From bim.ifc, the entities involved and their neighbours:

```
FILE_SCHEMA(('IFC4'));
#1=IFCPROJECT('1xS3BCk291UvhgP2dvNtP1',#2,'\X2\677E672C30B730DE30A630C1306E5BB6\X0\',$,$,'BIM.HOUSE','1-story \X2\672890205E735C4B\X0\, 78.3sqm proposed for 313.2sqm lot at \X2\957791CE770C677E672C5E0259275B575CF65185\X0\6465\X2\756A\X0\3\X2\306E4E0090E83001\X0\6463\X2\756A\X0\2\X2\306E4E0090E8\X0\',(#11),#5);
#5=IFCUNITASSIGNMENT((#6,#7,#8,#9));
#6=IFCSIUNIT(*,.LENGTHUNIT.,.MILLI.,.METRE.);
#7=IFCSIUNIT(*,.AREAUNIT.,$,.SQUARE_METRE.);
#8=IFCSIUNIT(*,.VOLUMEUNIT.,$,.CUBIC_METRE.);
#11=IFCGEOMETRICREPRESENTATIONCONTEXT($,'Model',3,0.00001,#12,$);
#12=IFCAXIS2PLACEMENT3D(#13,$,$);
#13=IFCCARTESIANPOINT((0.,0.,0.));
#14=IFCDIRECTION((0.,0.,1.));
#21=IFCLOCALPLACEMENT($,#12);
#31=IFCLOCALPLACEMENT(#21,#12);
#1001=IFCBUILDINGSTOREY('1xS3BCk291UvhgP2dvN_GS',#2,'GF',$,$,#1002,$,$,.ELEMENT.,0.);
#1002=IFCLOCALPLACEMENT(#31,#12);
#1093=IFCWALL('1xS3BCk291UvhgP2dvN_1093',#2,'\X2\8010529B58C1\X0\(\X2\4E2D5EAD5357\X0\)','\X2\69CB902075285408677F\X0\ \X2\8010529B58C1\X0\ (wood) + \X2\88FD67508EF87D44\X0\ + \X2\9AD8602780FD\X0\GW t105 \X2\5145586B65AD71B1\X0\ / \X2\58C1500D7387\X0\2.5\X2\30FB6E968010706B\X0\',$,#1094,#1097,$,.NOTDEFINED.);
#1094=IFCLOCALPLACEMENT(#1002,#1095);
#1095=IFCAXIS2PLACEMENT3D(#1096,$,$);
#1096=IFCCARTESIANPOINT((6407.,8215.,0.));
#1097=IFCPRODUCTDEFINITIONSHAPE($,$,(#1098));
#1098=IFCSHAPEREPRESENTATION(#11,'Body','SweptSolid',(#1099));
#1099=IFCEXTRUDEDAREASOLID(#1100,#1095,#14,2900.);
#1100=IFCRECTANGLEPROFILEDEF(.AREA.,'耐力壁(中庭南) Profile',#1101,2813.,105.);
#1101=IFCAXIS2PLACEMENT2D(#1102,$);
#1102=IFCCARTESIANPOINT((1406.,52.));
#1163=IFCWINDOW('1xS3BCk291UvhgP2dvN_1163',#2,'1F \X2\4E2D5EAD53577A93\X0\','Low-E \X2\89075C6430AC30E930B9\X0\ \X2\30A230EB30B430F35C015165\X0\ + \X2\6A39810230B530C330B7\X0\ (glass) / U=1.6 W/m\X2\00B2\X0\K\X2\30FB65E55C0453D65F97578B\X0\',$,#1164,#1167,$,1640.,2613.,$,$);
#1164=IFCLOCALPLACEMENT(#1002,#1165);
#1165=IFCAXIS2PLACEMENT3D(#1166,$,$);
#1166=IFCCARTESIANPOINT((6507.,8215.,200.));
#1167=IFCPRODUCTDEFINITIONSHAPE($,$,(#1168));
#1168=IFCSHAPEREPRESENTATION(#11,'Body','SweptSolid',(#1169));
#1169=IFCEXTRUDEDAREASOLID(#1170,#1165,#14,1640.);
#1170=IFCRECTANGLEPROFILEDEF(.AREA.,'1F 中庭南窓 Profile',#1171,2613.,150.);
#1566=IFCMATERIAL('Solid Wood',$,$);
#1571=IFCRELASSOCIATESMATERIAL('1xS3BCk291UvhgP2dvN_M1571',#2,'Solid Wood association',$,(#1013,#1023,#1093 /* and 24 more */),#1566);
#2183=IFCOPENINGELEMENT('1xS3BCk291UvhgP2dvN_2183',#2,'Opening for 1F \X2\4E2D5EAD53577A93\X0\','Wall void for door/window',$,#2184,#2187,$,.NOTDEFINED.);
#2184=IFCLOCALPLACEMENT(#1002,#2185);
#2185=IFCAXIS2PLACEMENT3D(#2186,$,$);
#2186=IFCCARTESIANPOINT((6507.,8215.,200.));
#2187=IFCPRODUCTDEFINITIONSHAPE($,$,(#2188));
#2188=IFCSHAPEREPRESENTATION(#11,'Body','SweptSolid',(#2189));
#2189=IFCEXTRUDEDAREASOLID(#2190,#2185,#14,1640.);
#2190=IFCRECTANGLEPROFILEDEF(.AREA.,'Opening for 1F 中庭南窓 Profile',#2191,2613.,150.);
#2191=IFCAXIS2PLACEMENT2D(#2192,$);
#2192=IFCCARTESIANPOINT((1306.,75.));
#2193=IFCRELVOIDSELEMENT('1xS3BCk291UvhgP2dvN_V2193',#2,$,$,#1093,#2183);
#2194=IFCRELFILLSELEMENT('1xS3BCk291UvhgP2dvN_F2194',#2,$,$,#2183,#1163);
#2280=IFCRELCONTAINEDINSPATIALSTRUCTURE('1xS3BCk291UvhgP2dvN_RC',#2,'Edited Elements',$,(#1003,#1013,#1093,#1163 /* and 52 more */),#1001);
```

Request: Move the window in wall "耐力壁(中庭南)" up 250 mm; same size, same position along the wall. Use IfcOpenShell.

```python
import numpy as np
import ifcopenshell
import ifcopenshell.api.geometry
import ifcopenshell.util.placement
import ifcopenshell.util.unit

model = ifcopenshell.open("bim.ifc")
unit_scale = ifcopenshell.util.unit.calculate_unit_scale(model)

window = model.by_guid("1xS3BCk291UvhgP2dvN_1163")
opening = window.FillsVoids[0].RelatingOpeningElement
dz = 250.0

shift = np.array([0.0, 0.0, dz])
# The window is not placed relative to its opening, so move both.
for product in (opening, window):
    matrix = ifcopenshell.util.placement.get_local_placement(product.ObjectPlacement)
    matrix[:3, 3] += shift
    ifcopenshell.api.geometry.edit_object_placement(model, product=product, matrix=matrix, is_si=False)

print(f"moved by {dz * unit_scale:+.3f} m")

model.write("bim_rev.ifc")
```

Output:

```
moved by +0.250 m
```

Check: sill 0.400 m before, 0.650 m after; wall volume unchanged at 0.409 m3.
